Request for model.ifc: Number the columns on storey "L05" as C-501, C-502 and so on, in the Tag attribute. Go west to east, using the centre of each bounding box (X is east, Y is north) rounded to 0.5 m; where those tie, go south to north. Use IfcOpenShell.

First a look at what the model holds.

```python
import ifcopenshell
import ifcopenshell.util.element
import ifcopenshell.util.placement

model = ifcopenshell.open("model.ifc")
print(model.schema)
storey = next(s for s in model.by_type("IfcBuildingStorey") if s.Name == "L05")
columns = [e for e in ifcopenshell.util.element.get_decomposition(storey) if e.is_a("IfcColumn")]
for e in sorted(columns, key=lambda e: e.id()):
    origin = ifcopenshell.util.placement.get_local_placement(e.ObjectPlacement)[:3, 3]
    print(e.id(), e.Tag, e.Name, origin.round(2) + 0.0, sep=" | ")
```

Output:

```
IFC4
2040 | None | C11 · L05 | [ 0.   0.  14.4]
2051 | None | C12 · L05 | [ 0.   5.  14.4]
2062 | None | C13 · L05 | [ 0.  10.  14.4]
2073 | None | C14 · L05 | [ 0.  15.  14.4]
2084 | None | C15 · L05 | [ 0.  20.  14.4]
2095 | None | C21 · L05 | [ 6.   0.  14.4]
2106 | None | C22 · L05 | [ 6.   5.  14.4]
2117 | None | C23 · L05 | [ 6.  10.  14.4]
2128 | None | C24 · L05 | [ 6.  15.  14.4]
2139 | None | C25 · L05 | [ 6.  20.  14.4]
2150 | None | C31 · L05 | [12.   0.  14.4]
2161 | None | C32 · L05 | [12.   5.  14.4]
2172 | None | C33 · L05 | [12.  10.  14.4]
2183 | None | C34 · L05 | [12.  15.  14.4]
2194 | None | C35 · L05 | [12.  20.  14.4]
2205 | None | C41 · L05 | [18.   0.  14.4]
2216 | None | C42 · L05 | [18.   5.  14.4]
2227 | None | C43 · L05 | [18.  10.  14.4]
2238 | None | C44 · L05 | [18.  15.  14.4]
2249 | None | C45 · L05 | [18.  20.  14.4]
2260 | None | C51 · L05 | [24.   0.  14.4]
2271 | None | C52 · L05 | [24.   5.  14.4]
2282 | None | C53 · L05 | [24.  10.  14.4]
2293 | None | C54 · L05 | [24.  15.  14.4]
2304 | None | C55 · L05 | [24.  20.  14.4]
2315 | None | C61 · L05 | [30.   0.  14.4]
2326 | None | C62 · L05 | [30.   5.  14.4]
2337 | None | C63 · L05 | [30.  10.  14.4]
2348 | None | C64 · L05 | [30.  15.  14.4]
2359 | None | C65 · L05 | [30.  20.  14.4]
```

```python
import ifcopenshell
import ifcopenshell.geom
import ifcopenshell.util.element
import ifcopenshell.util.shape

model = ifcopenshell.open("model.ifc")
settings = ifcopenshell.geom.settings()
settings.set("use-world-coords", True)


def centre(element):
    shape = ifcopenshell.geom.create_shape(settings, element)
    return ifcopenshell.util.shape.get_bbox_centroid(shape.geometry)


storey = next(s for s in model.by_type("IfcBuildingStorey") if s.Name == "L05")
columns = [e for e in ifcopenshell.util.element.get_decomposition(storey) if e.is_a("IfcColumn")]

# Insertion points can sit at a corner or the storey origin, so sort by the geometry (in metres).
centres = {e: centre(e) for e in columns}
columns.sort(key=lambda e: (round(centres[e][0] / 0.5), centres[e][1]))

for i, e in enumerate(columns, start=1):
    number = f"C-5{i:02d}"
    e.Tag = number
    print(e.id(), number)

model.write("model_updated.ifc")
```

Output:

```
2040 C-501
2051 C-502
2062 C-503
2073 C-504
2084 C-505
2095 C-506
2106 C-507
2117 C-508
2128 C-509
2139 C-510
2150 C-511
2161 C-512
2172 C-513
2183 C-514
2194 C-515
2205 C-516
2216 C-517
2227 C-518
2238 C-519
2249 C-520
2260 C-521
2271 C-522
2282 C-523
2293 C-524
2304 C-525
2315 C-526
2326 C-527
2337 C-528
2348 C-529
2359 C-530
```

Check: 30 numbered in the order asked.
